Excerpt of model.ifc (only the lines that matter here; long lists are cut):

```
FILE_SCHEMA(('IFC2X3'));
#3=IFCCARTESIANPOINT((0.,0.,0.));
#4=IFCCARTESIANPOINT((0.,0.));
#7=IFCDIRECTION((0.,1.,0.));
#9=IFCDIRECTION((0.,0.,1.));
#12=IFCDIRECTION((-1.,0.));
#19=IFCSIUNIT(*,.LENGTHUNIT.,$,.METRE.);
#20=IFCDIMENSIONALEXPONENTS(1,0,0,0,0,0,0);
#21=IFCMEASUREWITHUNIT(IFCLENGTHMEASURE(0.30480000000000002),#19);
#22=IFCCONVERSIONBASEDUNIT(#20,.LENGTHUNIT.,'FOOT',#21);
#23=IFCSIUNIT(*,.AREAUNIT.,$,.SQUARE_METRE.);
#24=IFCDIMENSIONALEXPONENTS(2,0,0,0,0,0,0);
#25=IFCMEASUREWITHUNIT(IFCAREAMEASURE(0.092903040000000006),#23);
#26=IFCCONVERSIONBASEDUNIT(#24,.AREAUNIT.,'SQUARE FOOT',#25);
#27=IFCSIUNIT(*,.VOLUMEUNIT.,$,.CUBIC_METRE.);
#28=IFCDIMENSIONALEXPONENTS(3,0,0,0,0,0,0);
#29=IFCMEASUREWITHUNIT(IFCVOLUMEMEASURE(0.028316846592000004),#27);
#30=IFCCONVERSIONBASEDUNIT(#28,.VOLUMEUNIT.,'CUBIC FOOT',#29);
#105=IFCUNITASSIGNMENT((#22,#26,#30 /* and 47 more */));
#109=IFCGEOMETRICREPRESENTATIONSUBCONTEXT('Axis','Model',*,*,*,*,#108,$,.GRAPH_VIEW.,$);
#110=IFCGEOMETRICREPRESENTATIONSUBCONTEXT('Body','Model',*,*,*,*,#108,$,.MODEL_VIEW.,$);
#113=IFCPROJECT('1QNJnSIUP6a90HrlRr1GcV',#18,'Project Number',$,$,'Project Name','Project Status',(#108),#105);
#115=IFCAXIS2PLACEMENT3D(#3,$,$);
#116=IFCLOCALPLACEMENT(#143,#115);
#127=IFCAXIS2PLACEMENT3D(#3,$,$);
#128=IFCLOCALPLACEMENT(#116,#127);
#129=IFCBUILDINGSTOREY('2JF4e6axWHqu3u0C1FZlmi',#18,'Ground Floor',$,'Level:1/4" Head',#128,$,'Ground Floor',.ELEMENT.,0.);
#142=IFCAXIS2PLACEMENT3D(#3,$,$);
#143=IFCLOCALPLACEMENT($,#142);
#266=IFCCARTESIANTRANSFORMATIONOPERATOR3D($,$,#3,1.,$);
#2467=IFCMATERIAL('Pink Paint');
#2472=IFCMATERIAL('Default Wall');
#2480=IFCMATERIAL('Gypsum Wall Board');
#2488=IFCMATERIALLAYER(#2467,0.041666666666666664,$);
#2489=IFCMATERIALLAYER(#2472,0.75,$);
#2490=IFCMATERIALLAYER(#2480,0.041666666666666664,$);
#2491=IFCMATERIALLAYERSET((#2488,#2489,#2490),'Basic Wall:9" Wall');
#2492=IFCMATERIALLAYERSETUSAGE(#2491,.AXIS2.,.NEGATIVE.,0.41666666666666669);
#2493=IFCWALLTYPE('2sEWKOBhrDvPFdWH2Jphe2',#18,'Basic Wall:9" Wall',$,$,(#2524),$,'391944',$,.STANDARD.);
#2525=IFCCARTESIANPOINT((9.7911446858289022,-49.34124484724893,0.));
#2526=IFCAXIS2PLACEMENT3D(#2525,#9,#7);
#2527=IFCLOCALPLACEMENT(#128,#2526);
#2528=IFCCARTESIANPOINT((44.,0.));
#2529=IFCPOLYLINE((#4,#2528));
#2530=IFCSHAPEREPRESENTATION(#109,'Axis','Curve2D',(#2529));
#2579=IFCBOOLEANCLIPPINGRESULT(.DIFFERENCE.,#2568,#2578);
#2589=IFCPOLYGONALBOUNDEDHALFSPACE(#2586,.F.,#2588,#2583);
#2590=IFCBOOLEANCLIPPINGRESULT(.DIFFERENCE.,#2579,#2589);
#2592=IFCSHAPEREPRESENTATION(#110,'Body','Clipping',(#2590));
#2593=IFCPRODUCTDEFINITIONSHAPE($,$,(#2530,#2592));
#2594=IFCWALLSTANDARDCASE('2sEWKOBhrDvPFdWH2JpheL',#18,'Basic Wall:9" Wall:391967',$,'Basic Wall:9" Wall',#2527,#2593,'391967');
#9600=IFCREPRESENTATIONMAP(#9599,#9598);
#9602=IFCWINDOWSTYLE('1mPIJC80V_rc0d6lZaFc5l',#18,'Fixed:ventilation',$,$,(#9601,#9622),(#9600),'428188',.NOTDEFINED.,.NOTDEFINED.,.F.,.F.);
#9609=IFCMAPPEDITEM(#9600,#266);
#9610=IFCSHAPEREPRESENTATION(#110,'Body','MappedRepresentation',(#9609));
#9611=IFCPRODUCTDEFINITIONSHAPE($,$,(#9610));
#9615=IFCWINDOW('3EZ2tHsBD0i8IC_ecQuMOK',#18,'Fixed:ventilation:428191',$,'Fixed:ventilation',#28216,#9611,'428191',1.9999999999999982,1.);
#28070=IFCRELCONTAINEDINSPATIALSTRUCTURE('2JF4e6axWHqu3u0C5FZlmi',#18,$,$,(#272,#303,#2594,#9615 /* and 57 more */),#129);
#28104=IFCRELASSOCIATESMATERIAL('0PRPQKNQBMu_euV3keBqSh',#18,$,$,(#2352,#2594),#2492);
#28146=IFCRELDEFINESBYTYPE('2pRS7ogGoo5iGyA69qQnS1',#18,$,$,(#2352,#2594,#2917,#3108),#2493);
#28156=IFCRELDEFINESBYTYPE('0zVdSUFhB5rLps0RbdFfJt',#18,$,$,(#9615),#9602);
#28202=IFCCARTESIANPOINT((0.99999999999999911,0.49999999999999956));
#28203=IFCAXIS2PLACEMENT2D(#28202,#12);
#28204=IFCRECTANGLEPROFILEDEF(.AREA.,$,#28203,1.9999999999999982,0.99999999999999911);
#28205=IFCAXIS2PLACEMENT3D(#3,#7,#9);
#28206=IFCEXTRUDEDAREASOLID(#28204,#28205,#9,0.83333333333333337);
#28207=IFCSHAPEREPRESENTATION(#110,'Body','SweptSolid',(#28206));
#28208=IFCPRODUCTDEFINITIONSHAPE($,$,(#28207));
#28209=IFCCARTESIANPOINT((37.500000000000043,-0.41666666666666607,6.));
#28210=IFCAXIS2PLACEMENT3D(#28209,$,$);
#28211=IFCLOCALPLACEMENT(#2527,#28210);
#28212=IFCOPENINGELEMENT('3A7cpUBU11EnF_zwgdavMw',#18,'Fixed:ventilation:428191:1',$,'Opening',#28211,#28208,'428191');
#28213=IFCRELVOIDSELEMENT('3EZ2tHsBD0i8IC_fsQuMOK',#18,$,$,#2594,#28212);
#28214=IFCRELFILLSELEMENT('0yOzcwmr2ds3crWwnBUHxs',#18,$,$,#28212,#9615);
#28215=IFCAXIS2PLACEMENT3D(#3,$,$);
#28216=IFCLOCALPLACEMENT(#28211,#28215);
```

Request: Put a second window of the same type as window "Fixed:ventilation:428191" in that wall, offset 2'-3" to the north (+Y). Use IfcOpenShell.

```python
import ifcopenshell
import ifcopenshell.api.feature
import ifcopenshell.api.geometry
import ifcopenshell.api.root
import ifcopenshell.geom
import ifcopenshell.util.element
import ifcopenshell.util.placement
import ifcopenshell.util.shape
import ifcopenshell.util.unit

model = ifcopenshell.open("model.ifc")
unit_scale = ifcopenshell.util.unit.calculate_unit_scale(model)
settings = ifcopenshell.geom.settings()


def volume(element):
    """Net volume in cubic metres, openings subtracted."""
    shape = ifcopenshell.geom.create_shape(settings, element)
    return ifcopenshell.util.shape.get_volume(shape.geometry)


def reuse_history(source, copy):
    """copy_class also copies each property set's owner history, people and application; keep the originals."""
    for rel in copy.IsDefinedBy:
        if rel.is_a("IfcRelDefinesByProperties") and (history := rel.RelatingPropertyDefinition.OwnerHistory):
            rel.RelatingPropertyDefinition.OwnerHistory = source.OwnerHistory
            ifcopenshell.util.element.remove_deep2(model, history)


window = model.by_guid("3EZ2tHsBD0i8IC_ecQuMOK")
opening = window.FillsVoids[0].RelatingOpeningElement
wall = opening.VoidsElements[0].RelatingBuildingElement
before = volume(wall)
shift = ifcopenshell.util.placement.get_local_placement(wall.ObjectPlacement)[:3, 0] * 27 * 0.0254 / unit_scale

# copy_class copies the void relationship, type, container and properties, but no geometry.
new_opening = ifcopenshell.api.root.copy_class(model, product=opening)
new_opening.Representation = ifcopenshell.util.element.copy_deep(
    model, opening.Representation, exclude=["IfcGeometricRepresentationContext", "IfcRepresentationMap"]
)
new_opening.Name = "Fixed:ventilation"
new_opening.Tag = None
new_window = ifcopenshell.api.root.copy_class(model, product=window)
new_window.Representation = ifcopenshell.util.element.copy_deep(
    model, window.Representation, exclude=["IfcGeometricRepresentationContext", "IfcRepresentationMap"]
)
new_window.Name = "Fixed:ventilation"
new_window.Tag = None
reuse_history(window, new_window)
fills = ifcopenshell.api.feature.add_filling(model, opening=new_opening, element=new_window)
fills.OwnerHistory = new_window.OwnerHistory  # required in IFC2X3

for old, new in ((opening, new_opening), (window, new_window)):
    matrix = ifcopenshell.util.placement.get_local_placement(old.ObjectPlacement)
    matrix[:3, 3] += shift
    ifcopenshell.api.geometry.edit_object_placement(model, product=new, matrix=matrix, is_si=False)

after = volume(wall)

print(f"wall volume {before:.3f} -> {after:.3f} m3")

model.write("model-out.ifc")
```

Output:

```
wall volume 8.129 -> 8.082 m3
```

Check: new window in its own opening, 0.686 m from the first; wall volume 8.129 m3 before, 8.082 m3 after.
